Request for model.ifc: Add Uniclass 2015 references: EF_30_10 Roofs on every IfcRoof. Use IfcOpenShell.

First a look at what the model holds.

```python
import ifcopenshell

model = ifcopenshell.open("model.ifc")
print(model.schema)
print("classifications:", [c.Name for c in model.by_type("IfcClassification")])
for ifc_class in ("IfcDoor", "IfcRoof", "IfcStair", "IfcWall", "IfcWindow"):
    print(ifc_class, len(model.by_type(ifc_class)))
```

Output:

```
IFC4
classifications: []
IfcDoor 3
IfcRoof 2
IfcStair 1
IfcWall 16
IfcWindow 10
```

```python
import ifcopenshell
import ifcopenshell.api.classification

model = ifcopenshell.open("model.ifc")

system = ifcopenshell.api.classification.add_classification(model, classification="Uniclass 2015")

codes = {
    "IfcRoof": ("EF_30_10", "Roofs"),
}
for ifc_class, (code, name) in codes.items():
    products = model.by_type(ifc_class)
    ifcopenshell.api.classification.add_reference(
        model, products=products, classification=system, identification=code, name=name
    )
    print(code, len(products))

model.write("model_updated.ifc")
```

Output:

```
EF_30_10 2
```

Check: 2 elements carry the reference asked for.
